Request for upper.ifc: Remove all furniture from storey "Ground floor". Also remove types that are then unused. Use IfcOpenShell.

First a look at what the model holds.

```python
import ifcopenshell
import ifcopenshell.util.element

model = ifcopenshell.open("upper.ifc")
print(model.schema)
storey = next(s for s in model.by_type("IfcBuildingStorey") if s.Name == "Ground floor")
furniture = [e for e in ifcopenshell.util.element.get_decomposition(storey) if e.is_a("IfcFurnishingElement")]
seen = {}
for e in furniture:
    element_type = ifcopenshell.util.element.get_type(e)
    name = element_type.Name if element_type not in (None, e) else None
    seen[name] = seen.get(name, 0) + 1
for name, count in sorted(seen.items(), key=str):
    print(count, "x", name)
```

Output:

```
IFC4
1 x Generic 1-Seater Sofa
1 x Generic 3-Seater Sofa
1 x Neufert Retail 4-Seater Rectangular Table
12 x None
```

```python
import ifcopenshell
import ifcopenshell.api.root
import ifcopenshell.util.element

model = ifcopenshell.open("upper.ifc")

storey = next(s for s in model.by_type("IfcBuildingStorey") if s.Name == "Ground floor")
furniture = [e for e in ifcopenshell.util.element.get_decomposition(storey) if e.is_a("IfcFurnishingElement")]
types = {ifcopenshell.util.element.get_type(e) for e in furniture} - {None, *furniture}

for e in furniture:
    ifcopenshell.api.root.remove_product(model, product=e)
print(len(furniture), "removed")

unused = [t for t in types if not ifcopenshell.util.element.get_types(t)]
for t in unused:
    ifcopenshell.api.root.remove_product(model, product=t)
print(len(unused), "unused types removed")

model.write("upper_updated.ifc")
```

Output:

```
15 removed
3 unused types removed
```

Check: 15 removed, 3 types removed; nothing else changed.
